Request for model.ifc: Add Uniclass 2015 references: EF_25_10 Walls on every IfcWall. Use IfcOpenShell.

First a look at what the model holds.

```python
import ifcopenshell

model = ifcopenshell.open("model.ifc")
print(model.schema)
print("classifications:", [c.Name for c in model.by_type("IfcClassification")])
for ifc_class in ("IfcDoor", "IfcRoof", "IfcStair", "IfcWall", "IfcWindow"):
    print(ifc_class, len(model.by_type(ifc_class)))
```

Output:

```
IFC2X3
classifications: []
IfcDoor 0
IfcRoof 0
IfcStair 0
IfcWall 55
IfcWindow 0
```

```python
import ifcopenshell
import ifcopenshell.api.classification

model = ifcopenshell.open("model.ifc")

# IFC2X3 requires Source and Edition and has no link from the project to the system.
system = model.create_entity("IfcClassification", Source="NBS", Edition="2015", Name="Uniclass 2015")

codes = {
    "IfcWall": ("EF_25_10", "Walls"),
}
for ifc_class, (code, name) in codes.items():
    products = model.by_type(ifc_class)
    ifcopenshell.api.classification.add_reference(
        model, products=products, classification=system, identification=code, name=name
    )
    print(code, len(products))

model.write("model_v2.ifc")
```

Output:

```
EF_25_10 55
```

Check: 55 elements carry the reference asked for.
